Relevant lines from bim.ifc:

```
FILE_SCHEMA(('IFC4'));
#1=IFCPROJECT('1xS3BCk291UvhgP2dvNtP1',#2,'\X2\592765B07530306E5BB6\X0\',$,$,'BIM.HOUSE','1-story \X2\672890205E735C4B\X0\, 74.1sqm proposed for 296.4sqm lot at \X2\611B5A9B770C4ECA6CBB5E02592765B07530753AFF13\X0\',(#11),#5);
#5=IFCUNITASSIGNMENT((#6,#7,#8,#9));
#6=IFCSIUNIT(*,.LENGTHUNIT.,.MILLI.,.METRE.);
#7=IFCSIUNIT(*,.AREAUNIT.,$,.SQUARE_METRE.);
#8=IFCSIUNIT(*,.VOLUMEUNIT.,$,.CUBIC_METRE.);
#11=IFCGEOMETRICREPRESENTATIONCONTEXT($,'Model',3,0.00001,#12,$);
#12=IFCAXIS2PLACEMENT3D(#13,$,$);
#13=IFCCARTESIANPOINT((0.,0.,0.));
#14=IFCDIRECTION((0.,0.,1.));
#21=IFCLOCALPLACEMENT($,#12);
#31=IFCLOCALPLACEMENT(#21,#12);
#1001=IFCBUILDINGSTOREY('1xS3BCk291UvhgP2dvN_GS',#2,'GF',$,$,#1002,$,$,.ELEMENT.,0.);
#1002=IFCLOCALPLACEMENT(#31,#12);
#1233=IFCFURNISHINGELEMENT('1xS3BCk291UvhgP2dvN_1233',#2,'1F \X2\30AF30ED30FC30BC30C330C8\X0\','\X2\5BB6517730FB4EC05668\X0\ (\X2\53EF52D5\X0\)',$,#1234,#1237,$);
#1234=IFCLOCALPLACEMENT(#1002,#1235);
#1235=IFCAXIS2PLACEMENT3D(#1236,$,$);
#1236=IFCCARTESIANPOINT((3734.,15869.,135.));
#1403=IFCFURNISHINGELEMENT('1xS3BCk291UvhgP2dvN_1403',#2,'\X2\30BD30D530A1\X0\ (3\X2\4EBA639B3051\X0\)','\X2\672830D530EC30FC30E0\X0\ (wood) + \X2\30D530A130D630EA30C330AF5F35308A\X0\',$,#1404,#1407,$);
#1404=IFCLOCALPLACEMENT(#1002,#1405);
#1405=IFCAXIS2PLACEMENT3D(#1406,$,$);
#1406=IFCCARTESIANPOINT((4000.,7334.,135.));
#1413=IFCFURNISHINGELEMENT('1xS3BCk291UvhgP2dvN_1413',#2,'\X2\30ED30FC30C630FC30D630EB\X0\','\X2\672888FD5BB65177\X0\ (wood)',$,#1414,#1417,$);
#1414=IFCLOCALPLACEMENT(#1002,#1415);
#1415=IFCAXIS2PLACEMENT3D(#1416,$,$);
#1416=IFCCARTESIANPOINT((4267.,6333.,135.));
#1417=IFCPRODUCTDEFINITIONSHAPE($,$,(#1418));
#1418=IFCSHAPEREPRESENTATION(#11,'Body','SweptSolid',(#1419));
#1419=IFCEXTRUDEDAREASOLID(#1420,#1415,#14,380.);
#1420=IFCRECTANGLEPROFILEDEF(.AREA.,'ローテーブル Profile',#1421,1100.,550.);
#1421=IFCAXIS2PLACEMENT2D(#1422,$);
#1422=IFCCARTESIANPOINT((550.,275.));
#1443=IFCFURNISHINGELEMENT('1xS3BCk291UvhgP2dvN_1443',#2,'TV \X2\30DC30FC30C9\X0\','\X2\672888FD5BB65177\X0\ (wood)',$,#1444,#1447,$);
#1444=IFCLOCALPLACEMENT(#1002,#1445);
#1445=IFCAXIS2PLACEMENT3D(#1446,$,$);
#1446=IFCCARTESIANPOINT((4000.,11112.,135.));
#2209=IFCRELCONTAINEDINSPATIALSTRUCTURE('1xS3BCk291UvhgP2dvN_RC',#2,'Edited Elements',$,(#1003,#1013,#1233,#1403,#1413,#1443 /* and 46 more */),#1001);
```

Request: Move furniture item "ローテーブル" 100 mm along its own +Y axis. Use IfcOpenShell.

```python
import ifcopenshell
import ifcopenshell.api.geometry
import ifcopenshell.util.placement

model = ifcopenshell.open("bim.ifc")

item = model.by_guid("1xS3BCk291UvhgP2dvN_1413")
matrix = ifcopenshell.util.placement.get_local_placement(item.ObjectPlacement)
matrix[:3, 3] += matrix[:3, 1] * 100.0
ifcopenshell.api.geometry.edit_object_placement(model, product=item, matrix=matrix, is_si=False)

print(ifcopenshell.util.placement.get_local_placement(item.ObjectPlacement).round(3) + 0.0)

model.write("bim_edited.ifc")
```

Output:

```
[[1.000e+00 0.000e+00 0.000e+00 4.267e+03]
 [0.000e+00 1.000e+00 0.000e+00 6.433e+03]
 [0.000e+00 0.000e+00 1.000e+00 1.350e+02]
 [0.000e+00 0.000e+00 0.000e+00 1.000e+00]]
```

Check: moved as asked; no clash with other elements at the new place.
